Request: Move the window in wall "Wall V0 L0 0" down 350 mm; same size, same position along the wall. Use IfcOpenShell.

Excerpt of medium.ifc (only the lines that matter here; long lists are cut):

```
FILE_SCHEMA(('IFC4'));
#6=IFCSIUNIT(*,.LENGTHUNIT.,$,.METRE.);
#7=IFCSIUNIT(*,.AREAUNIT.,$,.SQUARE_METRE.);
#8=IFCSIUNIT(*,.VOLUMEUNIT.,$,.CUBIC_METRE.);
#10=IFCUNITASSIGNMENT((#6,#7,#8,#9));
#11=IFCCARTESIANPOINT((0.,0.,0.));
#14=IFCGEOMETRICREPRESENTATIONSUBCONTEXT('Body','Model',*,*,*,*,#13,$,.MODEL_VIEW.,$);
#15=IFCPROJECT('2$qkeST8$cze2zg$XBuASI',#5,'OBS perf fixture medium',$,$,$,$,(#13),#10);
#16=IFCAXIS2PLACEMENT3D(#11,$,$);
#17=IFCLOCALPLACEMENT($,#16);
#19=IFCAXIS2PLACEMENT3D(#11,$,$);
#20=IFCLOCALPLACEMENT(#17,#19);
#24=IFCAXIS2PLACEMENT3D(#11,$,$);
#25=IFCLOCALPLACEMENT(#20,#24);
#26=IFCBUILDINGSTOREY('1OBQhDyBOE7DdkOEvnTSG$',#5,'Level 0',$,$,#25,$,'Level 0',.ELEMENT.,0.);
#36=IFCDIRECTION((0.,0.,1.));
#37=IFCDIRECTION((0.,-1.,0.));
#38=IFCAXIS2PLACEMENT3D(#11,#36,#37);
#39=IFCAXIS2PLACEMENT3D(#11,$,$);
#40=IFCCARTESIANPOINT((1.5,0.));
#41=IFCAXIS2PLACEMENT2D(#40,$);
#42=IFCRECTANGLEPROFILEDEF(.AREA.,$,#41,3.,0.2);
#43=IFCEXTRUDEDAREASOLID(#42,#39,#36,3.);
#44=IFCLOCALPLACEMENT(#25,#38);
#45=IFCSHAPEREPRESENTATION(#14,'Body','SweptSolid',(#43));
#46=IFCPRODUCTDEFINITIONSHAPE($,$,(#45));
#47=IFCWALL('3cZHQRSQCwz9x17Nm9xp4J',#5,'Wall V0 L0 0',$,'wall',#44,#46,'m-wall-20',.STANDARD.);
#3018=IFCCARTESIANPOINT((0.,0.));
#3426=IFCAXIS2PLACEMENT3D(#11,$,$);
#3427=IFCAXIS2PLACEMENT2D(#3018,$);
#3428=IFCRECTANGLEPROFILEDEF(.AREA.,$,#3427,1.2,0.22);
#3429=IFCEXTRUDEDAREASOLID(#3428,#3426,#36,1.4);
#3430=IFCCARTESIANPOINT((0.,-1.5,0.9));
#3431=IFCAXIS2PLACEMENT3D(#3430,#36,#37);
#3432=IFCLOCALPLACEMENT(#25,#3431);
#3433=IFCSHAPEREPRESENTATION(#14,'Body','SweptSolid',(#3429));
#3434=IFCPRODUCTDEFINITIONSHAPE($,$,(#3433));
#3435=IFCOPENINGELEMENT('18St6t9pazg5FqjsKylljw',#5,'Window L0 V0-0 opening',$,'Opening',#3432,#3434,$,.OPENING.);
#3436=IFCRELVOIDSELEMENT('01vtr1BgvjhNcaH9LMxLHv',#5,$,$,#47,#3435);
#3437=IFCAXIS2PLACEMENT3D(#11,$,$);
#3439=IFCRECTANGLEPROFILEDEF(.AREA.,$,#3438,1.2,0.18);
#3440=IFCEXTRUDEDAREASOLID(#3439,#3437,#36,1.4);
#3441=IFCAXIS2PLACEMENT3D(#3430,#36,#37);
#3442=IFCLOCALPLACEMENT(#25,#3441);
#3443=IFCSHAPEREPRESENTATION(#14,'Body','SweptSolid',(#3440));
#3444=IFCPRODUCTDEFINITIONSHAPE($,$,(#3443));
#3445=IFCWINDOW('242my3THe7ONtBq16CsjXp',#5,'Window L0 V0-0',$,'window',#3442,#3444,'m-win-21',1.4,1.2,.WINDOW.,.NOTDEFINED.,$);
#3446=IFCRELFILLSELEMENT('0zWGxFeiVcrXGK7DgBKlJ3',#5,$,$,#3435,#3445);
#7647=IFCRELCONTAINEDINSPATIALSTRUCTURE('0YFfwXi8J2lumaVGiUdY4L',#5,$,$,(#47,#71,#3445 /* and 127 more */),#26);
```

```python
import numpy as np
import ifcopenshell
import ifcopenshell.api.geometry
import ifcopenshell.util.placement
import ifcopenshell.util.unit

model = ifcopenshell.open("medium.ifc")
unit_scale = ifcopenshell.util.unit.calculate_unit_scale(model)

window = model.by_id(3445)
opening = window.FillsVoids[0].RelatingOpeningElement
dz = -0.35

shift = np.array([0.0, 0.0, dz])
# The window is not placed relative to its opening, so move both.
for product in (opening, window):
    matrix = ifcopenshell.util.placement.get_local_placement(product.ObjectPlacement)
    matrix[:3, 3] += shift
    ifcopenshell.api.geometry.edit_object_placement(model, product=product, matrix=matrix, is_si=False)

print(f"moved by {dz * unit_scale:+.3f} m")

model.write("medium_rev.ifc")
```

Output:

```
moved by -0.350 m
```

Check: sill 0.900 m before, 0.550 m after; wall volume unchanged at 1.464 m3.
